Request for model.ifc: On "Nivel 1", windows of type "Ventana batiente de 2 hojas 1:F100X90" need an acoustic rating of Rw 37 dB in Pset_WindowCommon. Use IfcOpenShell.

First a look at what the model holds.

```python
import ifcopenshell
import ifcopenshell.util.element

model = ifcopenshell.open("model.ifc")
print(model.schema)
storey = next(s for s in model.by_type("IfcBuildingStorey") if s.Name == "Nivel 1")
windows = [e for e in ifcopenshell.util.element.get_decomposition(storey) if e.is_a("IfcWindow")]
seen = {}
for e in windows:
    element_type = ifcopenshell.util.element.get_type(e)
    key = (element_type.Name if element_type != e and element_type else None, ifcopenshell.util.element.get_pset(e, "Pset_WindowCommon", "AcousticRating"))
    seen[key] = seen.get(key, 0) + 1
for (name, value), count in sorted(seen.items(), key=str):
    print(count, "x", name, "|", value)
```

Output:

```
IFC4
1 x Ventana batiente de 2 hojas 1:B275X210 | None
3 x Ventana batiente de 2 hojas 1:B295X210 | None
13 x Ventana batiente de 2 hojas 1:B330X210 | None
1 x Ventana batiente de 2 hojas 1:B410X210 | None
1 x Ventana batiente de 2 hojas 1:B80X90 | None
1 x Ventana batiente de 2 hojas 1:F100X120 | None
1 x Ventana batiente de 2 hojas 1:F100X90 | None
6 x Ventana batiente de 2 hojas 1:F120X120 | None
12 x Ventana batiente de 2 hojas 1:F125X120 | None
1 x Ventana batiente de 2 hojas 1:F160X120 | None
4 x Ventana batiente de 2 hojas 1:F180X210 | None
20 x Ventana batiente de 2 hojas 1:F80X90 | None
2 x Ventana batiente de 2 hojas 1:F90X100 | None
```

```python
import ifcopenshell
import ifcopenshell.api.pset
import ifcopenshell.util.element

model = ifcopenshell.open("model.ifc")

storey = next(s for s in model.by_type("IfcBuildingStorey") if s.Name == "Nivel 1")
windows = [e for e in ifcopenshell.util.element.get_decomposition(storey) if e.is_a("IfcWindow")]

count = 0
for e in windows:
    element_type = ifcopenshell.util.element.get_type(e)
    if element_type in (None, e) or element_type.Name != "Ventana batiente de 2 hojas 1:F100X90":
        continue
    # add_pset returns the element's existing set when there is one.
    pset = ifcopenshell.api.pset.add_pset(model, product=e, name="Pset_WindowCommon")
    ifcopenshell.api.pset.edit_pset(model, pset=pset, properties={"AcousticRating": "Rw 37 dB"})
    count += 1

print(count, "windows updated")

model.write("model_edited.ifc")
```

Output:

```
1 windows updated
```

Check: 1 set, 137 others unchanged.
